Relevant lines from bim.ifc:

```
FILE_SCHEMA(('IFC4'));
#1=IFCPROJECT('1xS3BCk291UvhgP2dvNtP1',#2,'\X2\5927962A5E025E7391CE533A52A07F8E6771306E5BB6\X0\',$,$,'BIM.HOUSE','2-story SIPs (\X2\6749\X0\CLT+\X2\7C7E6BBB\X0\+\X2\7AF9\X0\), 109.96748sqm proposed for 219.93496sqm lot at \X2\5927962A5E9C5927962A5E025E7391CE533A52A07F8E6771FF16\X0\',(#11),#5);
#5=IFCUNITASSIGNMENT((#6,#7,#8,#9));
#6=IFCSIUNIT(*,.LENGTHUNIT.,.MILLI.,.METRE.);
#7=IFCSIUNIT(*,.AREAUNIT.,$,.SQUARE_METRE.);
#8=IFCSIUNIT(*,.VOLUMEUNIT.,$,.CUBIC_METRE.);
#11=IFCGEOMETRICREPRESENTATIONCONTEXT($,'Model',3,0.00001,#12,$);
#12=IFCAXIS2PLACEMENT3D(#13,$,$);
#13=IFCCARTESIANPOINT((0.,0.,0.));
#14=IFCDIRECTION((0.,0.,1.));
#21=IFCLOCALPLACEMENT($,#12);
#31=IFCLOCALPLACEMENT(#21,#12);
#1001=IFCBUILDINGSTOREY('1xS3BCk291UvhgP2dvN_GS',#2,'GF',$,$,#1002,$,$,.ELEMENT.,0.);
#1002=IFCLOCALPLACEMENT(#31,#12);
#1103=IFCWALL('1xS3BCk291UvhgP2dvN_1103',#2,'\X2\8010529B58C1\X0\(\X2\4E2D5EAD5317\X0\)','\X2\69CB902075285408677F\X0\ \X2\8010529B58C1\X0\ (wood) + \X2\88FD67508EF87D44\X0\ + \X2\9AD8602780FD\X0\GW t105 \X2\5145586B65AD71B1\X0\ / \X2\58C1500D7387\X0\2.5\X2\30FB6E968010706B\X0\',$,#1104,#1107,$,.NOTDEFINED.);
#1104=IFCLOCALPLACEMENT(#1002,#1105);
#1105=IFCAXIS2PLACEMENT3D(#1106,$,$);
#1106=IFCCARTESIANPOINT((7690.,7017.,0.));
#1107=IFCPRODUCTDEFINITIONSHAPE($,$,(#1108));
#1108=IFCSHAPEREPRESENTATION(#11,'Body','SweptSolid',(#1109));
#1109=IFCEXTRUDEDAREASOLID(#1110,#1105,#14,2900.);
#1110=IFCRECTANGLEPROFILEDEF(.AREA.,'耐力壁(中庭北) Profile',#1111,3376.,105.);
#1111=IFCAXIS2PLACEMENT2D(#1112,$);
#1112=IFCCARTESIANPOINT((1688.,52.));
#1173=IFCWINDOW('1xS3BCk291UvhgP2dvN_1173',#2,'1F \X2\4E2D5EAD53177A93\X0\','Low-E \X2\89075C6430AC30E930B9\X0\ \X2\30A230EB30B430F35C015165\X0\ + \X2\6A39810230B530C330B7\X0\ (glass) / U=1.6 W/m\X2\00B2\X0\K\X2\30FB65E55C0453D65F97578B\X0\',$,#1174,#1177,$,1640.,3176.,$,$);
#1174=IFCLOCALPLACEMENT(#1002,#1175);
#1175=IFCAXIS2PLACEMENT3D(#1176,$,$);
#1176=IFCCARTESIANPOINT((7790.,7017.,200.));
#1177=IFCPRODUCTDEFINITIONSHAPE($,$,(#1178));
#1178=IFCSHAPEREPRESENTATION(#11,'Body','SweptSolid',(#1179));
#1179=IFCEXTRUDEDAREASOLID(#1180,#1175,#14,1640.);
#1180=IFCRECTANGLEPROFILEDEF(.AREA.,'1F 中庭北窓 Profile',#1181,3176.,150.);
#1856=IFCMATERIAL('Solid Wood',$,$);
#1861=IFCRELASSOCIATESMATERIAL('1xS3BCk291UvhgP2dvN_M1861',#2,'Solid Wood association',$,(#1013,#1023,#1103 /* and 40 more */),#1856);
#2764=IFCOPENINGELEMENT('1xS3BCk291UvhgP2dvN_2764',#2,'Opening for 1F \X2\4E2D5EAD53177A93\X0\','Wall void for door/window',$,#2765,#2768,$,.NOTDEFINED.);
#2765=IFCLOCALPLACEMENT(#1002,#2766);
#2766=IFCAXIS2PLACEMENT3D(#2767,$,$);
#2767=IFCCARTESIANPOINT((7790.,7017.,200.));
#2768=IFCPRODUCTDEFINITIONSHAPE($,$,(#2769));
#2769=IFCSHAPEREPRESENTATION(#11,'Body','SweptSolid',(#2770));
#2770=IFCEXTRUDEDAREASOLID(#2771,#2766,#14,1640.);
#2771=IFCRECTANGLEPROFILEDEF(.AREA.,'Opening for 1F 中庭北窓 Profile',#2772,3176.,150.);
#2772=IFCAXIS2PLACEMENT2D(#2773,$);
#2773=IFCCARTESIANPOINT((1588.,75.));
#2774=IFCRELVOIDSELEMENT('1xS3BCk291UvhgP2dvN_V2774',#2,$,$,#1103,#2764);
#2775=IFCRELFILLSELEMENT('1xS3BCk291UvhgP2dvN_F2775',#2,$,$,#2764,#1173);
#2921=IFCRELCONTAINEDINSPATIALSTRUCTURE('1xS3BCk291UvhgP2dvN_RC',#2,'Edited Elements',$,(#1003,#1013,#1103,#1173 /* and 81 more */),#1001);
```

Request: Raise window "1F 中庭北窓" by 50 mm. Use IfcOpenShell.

```python
import numpy as np
import ifcopenshell
import ifcopenshell.api.geometry
import ifcopenshell.util.placement
import ifcopenshell.util.unit

model = ifcopenshell.open("bim.ifc")
unit_scale = ifcopenshell.util.unit.calculate_unit_scale(model)

window = model.by_guid("1xS3BCk291UvhgP2dvN_1173")
opening = window.FillsVoids[0].RelatingOpeningElement
dz = 0.05 / unit_scale

shift = np.array([0.0, 0.0, dz])
# The window is not placed relative to its opening, so move both.
for product in (opening, window):
    matrix = ifcopenshell.util.placement.get_local_placement(product.ObjectPlacement)
    matrix[:3, 3] += shift
    ifcopenshell.api.geometry.edit_object_placement(model, product=product, matrix=matrix, is_si=False)

print(f"moved by {dz * unit_scale:+.3f} m")

model.write("bim_edited.ifc")
```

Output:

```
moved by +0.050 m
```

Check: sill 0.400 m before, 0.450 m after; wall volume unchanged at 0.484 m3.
